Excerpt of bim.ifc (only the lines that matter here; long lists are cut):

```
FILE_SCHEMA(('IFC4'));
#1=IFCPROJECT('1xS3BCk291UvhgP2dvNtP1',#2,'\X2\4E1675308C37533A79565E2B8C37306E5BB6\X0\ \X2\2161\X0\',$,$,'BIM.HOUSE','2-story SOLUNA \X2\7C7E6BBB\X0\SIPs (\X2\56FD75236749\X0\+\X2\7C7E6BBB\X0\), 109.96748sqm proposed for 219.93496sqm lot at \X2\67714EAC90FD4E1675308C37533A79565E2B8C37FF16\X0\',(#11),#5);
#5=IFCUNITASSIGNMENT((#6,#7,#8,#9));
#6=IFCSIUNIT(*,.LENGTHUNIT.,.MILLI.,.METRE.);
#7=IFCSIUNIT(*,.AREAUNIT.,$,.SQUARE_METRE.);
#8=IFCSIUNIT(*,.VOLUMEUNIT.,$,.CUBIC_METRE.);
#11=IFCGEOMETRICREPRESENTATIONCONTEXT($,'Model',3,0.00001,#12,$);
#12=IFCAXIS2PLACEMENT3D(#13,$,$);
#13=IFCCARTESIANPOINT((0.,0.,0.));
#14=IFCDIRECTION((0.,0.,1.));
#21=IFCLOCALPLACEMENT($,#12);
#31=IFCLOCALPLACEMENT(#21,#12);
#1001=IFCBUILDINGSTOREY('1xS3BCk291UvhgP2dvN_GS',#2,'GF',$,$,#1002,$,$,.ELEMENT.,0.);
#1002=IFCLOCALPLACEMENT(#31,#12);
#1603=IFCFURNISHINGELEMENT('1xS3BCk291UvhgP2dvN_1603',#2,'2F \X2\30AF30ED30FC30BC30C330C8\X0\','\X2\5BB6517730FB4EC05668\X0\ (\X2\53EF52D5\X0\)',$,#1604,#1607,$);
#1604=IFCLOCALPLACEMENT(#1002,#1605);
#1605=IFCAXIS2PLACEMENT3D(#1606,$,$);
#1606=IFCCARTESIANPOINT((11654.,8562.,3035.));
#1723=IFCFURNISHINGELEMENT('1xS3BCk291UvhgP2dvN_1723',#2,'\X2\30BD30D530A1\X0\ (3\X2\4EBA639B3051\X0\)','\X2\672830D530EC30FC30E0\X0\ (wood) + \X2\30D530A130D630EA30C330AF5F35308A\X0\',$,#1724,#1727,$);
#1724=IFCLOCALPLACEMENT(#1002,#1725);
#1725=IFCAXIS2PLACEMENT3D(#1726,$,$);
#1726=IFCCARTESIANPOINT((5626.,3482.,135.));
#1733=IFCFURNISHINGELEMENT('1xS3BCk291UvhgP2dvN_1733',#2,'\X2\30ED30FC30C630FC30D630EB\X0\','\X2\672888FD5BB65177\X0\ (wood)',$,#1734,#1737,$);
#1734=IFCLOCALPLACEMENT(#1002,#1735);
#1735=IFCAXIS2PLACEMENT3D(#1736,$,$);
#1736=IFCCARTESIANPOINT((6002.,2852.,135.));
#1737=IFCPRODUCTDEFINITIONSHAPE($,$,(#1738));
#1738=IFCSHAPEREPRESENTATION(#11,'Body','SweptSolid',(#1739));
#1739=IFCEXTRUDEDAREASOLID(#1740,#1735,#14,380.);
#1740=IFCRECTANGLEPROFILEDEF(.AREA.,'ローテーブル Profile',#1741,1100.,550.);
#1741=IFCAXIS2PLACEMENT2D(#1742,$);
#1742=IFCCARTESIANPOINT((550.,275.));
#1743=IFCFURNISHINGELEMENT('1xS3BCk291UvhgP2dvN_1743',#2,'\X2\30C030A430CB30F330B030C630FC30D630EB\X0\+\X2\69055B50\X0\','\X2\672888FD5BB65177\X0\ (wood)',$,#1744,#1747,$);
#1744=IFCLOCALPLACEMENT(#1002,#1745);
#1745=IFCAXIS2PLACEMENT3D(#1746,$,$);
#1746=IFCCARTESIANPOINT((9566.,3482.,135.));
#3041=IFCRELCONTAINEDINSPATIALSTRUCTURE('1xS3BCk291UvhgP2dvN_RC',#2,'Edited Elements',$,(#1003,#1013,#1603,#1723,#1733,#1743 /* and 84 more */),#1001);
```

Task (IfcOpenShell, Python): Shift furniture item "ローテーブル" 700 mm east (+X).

```python
import ifcopenshell
import ifcopenshell.api.geometry
import ifcopenshell.util.placement
import ifcopenshell.util.unit

model = ifcopenshell.open("bim.ifc")
unit_scale = ifcopenshell.util.unit.calculate_unit_scale(model)

item = model.by_guid("1xS3BCk291UvhgP2dvN_1733")
matrix = ifcopenshell.util.placement.get_local_placement(item.ObjectPlacement)
matrix[0, 3] += 0.7 / unit_scale
ifcopenshell.api.geometry.edit_object_placement(model, product=item, matrix=matrix, is_si=False)

print(ifcopenshell.util.placement.get_local_placement(item.ObjectPlacement).round(3) + 0.0)

model.write("bim_edited.ifc")
```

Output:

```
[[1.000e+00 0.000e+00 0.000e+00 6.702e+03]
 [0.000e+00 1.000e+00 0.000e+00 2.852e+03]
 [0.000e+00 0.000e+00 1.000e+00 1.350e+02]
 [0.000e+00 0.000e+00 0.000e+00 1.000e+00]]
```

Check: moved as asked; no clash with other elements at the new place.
